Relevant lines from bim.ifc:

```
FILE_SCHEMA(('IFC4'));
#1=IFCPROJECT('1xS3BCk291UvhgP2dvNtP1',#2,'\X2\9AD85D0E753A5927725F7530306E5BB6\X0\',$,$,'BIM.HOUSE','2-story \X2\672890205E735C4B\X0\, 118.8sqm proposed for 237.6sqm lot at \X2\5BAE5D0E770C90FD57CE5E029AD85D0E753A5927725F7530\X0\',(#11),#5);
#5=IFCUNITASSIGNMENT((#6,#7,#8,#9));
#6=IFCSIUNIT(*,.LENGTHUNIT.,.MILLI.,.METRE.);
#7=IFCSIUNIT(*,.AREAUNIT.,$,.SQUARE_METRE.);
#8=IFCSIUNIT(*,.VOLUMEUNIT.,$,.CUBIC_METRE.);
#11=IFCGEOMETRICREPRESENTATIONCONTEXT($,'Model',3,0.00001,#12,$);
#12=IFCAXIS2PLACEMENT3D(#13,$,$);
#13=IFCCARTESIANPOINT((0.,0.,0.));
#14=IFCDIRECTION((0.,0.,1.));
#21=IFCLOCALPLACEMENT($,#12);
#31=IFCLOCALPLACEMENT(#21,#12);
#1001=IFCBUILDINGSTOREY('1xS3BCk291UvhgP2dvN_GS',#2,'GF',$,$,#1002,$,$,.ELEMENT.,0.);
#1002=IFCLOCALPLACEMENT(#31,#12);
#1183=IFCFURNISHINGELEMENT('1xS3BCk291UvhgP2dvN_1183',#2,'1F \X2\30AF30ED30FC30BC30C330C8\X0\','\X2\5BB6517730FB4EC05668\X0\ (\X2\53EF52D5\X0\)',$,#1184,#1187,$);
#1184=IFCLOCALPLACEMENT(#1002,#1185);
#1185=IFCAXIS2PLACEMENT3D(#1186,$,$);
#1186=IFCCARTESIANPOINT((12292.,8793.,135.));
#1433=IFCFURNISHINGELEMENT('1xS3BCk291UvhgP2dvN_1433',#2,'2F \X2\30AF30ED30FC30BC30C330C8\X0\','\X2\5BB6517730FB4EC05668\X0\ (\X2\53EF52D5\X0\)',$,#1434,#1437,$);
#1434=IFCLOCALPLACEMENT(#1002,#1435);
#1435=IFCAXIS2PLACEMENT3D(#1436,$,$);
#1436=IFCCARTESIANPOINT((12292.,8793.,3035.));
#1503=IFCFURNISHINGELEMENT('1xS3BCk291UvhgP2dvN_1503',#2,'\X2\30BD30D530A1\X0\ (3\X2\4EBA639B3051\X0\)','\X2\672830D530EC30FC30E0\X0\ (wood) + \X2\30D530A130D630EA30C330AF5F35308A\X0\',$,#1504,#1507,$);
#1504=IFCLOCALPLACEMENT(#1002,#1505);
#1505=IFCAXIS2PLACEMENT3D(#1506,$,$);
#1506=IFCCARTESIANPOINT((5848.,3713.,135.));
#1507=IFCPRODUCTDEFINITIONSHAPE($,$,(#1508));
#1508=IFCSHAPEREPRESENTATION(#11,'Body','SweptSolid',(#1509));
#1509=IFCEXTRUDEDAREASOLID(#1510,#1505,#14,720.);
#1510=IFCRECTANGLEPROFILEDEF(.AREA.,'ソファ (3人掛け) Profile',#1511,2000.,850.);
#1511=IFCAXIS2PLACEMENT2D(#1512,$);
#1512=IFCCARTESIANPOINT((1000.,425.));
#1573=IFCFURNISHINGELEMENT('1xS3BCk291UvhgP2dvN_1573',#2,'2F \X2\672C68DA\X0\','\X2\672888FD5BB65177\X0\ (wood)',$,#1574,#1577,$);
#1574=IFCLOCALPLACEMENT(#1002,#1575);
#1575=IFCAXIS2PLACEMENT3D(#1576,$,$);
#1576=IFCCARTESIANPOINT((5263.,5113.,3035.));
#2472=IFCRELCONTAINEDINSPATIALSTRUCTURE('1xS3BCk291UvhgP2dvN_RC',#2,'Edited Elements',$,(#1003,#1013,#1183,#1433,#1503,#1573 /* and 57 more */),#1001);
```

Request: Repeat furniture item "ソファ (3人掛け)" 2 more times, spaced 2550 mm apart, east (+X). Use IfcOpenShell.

```python
import numpy as np
import ifcopenshell
import ifcopenshell.api.geometry
import ifcopenshell.api.root
import ifcopenshell.util.element
import ifcopenshell.util.placement

model = ifcopenshell.open("bim.ifc")


def reuse_history(source, copy):
    """copy_class also copies each property set's owner history, people and application; keep the originals."""
    for rel in copy.IsDefinedBy:
        if rel.is_a("IfcRelDefinesByProperties") and (history := rel.RelatingPropertyDefinition.OwnerHistory):
            rel.RelatingPropertyDefinition.OwnerHistory = source.OwnerHistory
            ifcopenshell.util.element.remove_deep2(model, history)


source = model.by_guid("1xS3BCk291UvhgP2dvN_1503")
base = ifcopenshell.util.placement.get_local_placement(source.ObjectPlacement)
step = np.array([1.0, 0.0, 0.0]) * 2550.0

for i in range(1, 3):
    copy = ifcopenshell.api.root.copy_class(model, product=source)
    copy.Representation = ifcopenshell.util.element.copy_deep(
        model, source.Representation, exclude=["IfcGeometricRepresentationContext", "IfcRepresentationMap"]
    )
    reuse_history(source, copy)
    matrix = base.copy()
    matrix[:3, 3] += i * step
    print("added at", matrix[:3, 3].round(3) + 0.0)
    ifcopenshell.api.geometry.edit_object_placement(model, product=copy, matrix=matrix, is_si=False)

model.write("bim_edited.ifc")
```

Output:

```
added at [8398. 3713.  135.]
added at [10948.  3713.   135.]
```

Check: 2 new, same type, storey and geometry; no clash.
